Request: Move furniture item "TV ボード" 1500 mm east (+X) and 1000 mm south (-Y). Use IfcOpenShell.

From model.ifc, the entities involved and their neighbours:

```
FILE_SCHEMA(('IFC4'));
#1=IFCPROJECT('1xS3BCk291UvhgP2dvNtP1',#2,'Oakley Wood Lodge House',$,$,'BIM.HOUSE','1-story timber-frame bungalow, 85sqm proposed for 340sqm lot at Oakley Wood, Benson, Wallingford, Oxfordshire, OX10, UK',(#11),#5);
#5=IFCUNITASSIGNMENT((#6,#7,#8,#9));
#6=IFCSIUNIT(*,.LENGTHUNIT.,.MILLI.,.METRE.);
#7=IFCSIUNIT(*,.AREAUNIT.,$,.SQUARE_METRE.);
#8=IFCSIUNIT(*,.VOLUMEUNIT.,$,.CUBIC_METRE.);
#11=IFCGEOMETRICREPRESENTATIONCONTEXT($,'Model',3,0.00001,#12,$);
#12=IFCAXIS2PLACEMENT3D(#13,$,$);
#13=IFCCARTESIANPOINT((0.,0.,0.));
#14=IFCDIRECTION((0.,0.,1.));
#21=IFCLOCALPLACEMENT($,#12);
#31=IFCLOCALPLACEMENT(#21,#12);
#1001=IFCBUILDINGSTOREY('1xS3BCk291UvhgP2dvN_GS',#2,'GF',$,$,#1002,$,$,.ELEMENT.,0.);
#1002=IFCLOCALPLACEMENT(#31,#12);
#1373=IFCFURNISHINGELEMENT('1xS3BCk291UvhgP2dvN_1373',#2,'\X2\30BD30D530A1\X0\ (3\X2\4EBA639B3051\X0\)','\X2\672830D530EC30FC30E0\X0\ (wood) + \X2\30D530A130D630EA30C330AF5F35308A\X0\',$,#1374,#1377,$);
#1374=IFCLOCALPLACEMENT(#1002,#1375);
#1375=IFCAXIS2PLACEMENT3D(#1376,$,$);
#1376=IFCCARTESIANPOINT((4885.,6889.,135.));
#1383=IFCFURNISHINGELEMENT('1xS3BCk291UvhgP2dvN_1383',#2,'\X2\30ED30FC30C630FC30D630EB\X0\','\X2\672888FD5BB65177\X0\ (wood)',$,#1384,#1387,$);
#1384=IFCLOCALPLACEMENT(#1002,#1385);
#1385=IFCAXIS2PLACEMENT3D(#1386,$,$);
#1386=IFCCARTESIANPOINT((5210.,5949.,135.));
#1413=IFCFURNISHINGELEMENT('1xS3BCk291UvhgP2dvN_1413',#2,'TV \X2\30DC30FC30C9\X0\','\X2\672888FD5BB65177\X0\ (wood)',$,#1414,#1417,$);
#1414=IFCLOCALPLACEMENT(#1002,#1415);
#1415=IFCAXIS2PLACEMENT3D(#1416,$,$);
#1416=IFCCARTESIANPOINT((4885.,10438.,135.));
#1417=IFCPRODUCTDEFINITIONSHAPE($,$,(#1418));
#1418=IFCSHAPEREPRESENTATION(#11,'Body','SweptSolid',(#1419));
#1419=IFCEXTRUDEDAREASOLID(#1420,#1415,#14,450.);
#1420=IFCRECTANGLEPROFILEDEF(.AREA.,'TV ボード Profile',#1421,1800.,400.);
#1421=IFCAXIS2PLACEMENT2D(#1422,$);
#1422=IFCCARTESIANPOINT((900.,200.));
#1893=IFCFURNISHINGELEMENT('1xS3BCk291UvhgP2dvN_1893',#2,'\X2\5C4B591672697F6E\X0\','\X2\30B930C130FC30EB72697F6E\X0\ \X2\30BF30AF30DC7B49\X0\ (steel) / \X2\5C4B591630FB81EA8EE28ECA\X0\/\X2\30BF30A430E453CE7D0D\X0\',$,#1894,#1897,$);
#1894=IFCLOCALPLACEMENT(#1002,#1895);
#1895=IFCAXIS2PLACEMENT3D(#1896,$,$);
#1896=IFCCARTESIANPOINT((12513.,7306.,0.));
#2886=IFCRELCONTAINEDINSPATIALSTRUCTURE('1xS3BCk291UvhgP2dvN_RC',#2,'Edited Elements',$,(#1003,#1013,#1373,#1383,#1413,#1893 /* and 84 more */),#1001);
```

```python
import ifcopenshell
import ifcopenshell.api.geometry
import ifcopenshell.util.placement
import ifcopenshell.util.unit

model = ifcopenshell.open("model.ifc")
unit_scale = ifcopenshell.util.unit.calculate_unit_scale(model)

item = model.by_id(1413)
matrix = ifcopenshell.util.placement.get_local_placement(item.ObjectPlacement)
matrix[0, 3] += 1.5 / unit_scale
matrix[1, 3] -= 1 / unit_scale
ifcopenshell.api.geometry.edit_object_placement(model, product=item, matrix=matrix, is_si=False)

print(ifcopenshell.util.placement.get_local_placement(item.ObjectPlacement).round(3) + 0.0)

model.write("model-out.ifc")
```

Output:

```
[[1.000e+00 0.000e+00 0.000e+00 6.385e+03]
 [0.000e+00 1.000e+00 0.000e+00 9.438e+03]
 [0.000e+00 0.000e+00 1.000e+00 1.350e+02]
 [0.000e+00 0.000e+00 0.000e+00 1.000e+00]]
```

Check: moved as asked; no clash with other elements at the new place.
